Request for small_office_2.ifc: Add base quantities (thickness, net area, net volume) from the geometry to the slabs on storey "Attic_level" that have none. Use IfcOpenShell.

First a look at what the model holds.

```python
import ifcopenshell
import ifcopenshell.util.element
import ifcopenshell.util.unit

model = ifcopenshell.open("small_office_2.ifc")
print(model.schema)
for unit_type in ("LENGTHUNIT", "AREAUNIT", "VOLUMEUNIT"):
    print(unit_type, ifcopenshell.util.unit.calculate_unit_scale(model, unit_type))
storey = next(s for s in model.by_type("IfcBuildingStorey") if s.Name == "Attic_level")
slabs = [e for e in ifcopenshell.util.element.get_decomposition(storey) if e.is_a("IfcSlab")]
for e in sorted(slabs, key=lambda e: e.id()):
    print(e.id(), e.is_a(), e.Name, list(ifcopenshell.util.element.get_psets(e, qtos_only=True)), sep=" | ")
```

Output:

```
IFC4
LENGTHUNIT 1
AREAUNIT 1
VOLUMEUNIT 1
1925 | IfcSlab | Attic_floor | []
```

```python
import ifcopenshell
import ifcopenshell.api.pset
import ifcopenshell.geom
import ifcopenshell.util.element
import ifcopenshell.util.shape
import ifcopenshell.util.unit

model = ifcopenshell.open("small_office_2.ifc")
unit_scale = ifcopenshell.util.unit.calculate_unit_scale(model)
area_scale = ifcopenshell.util.unit.calculate_unit_scale(model, "AREAUNIT")
volume_scale = ifcopenshell.util.unit.calculate_unit_scale(model, "VOLUMEUNIT")
settings = ifcopenshell.geom.settings()

storey = next(s for s in model.by_type("IfcBuildingStorey") if s.Name == "Attic_level")
slabs = [e for e in ifcopenshell.util.element.get_decomposition(storey) if e.is_a("IfcSlab")]

for e in sorted(slabs, key=lambda e: e.id()):
    if ifcopenshell.util.element.get_psets(e, qtos_only=True, should_inherit=False):
        continue
    # Geometry comes back in metres, in the element's own axes.
    shape = ifcopenshell.geom.create_shape(settings, e)
    values = {
        "Width": ifcopenshell.util.shape.get_z(shape.geometry) / unit_scale,
        "NetArea": ifcopenshell.util.shape.get_footprint_area(shape.geometry) / area_scale,
        "NetVolume": ifcopenshell.util.shape.get_volume(shape.geometry) / volume_scale,
    }
    qto = ifcopenshell.api.pset.add_qto(model, product=e, name="Qto_SlabBaseQuantities")
    ifcopenshell.api.pset.edit_qto(model, qto=qto, properties=values)
    print(e.id(), {k: round(v, 3) for k, v in values.items()})

model.write("small_office_2_edited.ifc")
```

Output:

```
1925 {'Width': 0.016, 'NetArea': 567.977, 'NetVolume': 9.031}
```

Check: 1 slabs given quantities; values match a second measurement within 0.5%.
